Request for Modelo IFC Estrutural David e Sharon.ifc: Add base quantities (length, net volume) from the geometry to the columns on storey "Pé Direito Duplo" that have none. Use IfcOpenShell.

First a look at what the model holds.

```python
import ifcopenshell
import ifcopenshell.util.element
import ifcopenshell.util.unit

model = ifcopenshell.open("Modelo IFC Estrutural David e Sharon.ifc")
print(model.schema)
for unit_type in ("LENGTHUNIT", "AREAUNIT", "VOLUMEUNIT"):
    print(unit_type, ifcopenshell.util.unit.calculate_unit_scale(model, unit_type))
storey = next(s for s in model.by_type("IfcBuildingStorey") if s.Name == "Pé Direito Duplo")
columns = [e for e in ifcopenshell.util.element.get_decomposition(storey) if e.is_a("IfcColumn")]
for e in sorted(columns, key=lambda e: e.id()):
    print(e.id(), e.is_a(), e.Name, list(ifcopenshell.util.element.get_psets(e, qtos_only=True)), sep=" | ")
```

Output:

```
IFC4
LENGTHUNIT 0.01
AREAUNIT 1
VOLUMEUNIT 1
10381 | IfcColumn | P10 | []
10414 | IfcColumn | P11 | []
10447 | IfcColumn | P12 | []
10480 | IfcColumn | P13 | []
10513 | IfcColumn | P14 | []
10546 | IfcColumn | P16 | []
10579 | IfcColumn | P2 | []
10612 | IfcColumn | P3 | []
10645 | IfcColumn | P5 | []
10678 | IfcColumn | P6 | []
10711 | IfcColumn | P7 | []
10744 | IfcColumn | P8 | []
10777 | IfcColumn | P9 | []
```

```python
import ifcopenshell
import ifcopenshell.api.pset
import ifcopenshell.geom
import ifcopenshell.util.element
import ifcopenshell.util.shape
import ifcopenshell.util.unit

model = ifcopenshell.open("Modelo IFC Estrutural David e Sharon.ifc")
unit_scale = ifcopenshell.util.unit.calculate_unit_scale(model)
volume_scale = ifcopenshell.util.unit.calculate_unit_scale(model, "VOLUMEUNIT")
settings = ifcopenshell.geom.settings()

storey = next(s for s in model.by_type("IfcBuildingStorey") if s.Name == "Pé Direito Duplo")
columns = [e for e in ifcopenshell.util.element.get_decomposition(storey) if e.is_a("IfcColumn")]

for e in sorted(columns, key=lambda e: e.id()):
    if ifcopenshell.util.element.get_psets(e, qtos_only=True, should_inherit=False):
        continue
    # Geometry comes back in metres, in the element's own axes.
    shape = ifcopenshell.geom.create_shape(settings, e)
    values = {
        "Length": ifcopenshell.util.shape.get_z(shape.geometry) / unit_scale,
        "NetVolume": ifcopenshell.util.shape.get_volume(shape.geometry) / volume_scale,
    }
    qto = ifcopenshell.api.pset.add_qto(model, product=e, name="Qto_ColumnBaseQuantities")
    ifcopenshell.api.pset.edit_qto(model, qto=qto, properties=values)
    print(e.id(), {k: round(v, 3) for k, v in values.items()})

model.write("Modelo IFC Estrutural David e Sharon_v2.ifc")
```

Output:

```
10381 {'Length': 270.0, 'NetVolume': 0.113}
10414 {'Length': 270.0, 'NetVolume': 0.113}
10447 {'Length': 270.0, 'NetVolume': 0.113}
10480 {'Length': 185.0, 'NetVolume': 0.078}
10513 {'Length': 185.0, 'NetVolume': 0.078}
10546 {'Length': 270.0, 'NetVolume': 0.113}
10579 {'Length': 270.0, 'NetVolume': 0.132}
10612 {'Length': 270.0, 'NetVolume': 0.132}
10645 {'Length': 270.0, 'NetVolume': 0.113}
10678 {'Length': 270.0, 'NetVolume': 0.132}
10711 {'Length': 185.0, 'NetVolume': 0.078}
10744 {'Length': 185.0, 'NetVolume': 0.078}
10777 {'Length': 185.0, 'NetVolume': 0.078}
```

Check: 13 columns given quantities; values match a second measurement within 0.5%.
